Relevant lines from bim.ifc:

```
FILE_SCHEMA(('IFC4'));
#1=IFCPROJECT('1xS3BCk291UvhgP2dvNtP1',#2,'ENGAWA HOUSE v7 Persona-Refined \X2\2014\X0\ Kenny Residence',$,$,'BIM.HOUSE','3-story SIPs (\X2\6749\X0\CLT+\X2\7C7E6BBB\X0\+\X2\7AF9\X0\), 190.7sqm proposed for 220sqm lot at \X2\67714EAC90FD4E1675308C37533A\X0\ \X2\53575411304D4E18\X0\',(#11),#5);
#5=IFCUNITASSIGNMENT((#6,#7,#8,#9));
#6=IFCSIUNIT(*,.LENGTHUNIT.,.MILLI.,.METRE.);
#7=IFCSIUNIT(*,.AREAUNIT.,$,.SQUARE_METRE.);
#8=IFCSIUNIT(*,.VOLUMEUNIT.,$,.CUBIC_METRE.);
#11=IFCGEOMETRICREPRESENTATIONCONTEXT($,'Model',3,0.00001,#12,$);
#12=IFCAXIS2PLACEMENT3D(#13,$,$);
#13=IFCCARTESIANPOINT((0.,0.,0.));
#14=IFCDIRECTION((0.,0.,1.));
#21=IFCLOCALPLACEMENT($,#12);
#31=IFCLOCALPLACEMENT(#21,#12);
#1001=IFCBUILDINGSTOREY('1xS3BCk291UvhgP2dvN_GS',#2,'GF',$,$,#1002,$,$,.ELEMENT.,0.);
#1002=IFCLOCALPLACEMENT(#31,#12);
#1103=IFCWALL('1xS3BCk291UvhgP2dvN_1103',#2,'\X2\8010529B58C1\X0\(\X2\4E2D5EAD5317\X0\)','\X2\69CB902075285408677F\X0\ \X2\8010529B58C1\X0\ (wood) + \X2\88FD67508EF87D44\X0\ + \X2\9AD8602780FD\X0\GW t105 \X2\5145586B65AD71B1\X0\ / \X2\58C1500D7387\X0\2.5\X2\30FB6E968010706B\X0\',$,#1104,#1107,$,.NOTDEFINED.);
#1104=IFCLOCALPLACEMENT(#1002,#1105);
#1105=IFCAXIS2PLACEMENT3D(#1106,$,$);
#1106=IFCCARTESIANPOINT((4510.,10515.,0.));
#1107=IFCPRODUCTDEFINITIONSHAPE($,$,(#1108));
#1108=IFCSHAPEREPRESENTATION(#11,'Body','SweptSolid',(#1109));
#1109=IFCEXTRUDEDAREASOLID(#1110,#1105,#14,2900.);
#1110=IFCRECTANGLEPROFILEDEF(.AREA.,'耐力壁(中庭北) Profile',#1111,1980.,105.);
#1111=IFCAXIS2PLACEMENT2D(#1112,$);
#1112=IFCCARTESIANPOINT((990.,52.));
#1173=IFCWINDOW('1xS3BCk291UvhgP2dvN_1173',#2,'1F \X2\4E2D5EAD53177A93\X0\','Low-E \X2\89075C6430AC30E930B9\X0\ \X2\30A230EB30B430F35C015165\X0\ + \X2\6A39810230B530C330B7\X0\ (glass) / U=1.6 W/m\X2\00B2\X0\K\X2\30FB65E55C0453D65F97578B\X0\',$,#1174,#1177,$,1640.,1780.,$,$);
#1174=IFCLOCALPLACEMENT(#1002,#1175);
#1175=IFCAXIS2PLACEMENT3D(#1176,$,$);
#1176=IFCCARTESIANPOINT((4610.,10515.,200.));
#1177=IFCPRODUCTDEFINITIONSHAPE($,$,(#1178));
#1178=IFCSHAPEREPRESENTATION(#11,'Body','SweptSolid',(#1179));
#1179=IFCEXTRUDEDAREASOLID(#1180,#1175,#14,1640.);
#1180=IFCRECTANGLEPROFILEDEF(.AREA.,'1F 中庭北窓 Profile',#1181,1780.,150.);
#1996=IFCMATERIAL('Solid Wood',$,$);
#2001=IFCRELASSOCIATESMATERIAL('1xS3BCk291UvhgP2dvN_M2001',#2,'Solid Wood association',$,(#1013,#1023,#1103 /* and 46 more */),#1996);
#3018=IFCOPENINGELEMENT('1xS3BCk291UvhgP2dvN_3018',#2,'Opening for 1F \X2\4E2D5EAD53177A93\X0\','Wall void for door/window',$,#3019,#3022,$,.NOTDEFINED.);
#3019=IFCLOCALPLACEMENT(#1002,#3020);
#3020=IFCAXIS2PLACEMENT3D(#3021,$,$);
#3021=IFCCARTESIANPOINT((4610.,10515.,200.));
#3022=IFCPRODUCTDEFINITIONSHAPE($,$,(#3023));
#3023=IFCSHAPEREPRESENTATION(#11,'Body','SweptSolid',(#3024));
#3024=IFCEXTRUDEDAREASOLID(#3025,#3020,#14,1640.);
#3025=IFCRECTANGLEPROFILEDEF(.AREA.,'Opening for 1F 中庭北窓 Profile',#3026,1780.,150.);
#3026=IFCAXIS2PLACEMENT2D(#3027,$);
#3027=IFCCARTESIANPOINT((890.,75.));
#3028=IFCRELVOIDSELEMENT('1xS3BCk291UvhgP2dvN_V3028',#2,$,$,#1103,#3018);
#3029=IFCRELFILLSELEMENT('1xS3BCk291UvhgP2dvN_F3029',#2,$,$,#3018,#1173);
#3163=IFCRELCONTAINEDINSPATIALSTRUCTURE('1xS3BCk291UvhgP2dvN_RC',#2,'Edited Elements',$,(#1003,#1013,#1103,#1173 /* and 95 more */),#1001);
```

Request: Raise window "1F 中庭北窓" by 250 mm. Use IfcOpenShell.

```python
import numpy as np
import ifcopenshell
import ifcopenshell.api.geometry
import ifcopenshell.util.placement
import ifcopenshell.util.unit

model = ifcopenshell.open("bim.ifc")
unit_scale = ifcopenshell.util.unit.calculate_unit_scale(model)

window = model.by_guid("1xS3BCk291UvhgP2dvN_1173")
opening = window.FillsVoids[0].RelatingOpeningElement
dz = 250.0

shift = np.array([0.0, 0.0, dz])
# The window is not placed relative to its opening, so move both.
for product in (opening, window):
    matrix = ifcopenshell.util.placement.get_local_placement(product.ObjectPlacement)
    matrix[:3, 3] += shift
    ifcopenshell.api.geometry.edit_object_placement(model, product=product, matrix=matrix, is_si=False)

print(f"moved by {dz * unit_scale:+.3f} m")

model.write("bim_edited.ifc")
```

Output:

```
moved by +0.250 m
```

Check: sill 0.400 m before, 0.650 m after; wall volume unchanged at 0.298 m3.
